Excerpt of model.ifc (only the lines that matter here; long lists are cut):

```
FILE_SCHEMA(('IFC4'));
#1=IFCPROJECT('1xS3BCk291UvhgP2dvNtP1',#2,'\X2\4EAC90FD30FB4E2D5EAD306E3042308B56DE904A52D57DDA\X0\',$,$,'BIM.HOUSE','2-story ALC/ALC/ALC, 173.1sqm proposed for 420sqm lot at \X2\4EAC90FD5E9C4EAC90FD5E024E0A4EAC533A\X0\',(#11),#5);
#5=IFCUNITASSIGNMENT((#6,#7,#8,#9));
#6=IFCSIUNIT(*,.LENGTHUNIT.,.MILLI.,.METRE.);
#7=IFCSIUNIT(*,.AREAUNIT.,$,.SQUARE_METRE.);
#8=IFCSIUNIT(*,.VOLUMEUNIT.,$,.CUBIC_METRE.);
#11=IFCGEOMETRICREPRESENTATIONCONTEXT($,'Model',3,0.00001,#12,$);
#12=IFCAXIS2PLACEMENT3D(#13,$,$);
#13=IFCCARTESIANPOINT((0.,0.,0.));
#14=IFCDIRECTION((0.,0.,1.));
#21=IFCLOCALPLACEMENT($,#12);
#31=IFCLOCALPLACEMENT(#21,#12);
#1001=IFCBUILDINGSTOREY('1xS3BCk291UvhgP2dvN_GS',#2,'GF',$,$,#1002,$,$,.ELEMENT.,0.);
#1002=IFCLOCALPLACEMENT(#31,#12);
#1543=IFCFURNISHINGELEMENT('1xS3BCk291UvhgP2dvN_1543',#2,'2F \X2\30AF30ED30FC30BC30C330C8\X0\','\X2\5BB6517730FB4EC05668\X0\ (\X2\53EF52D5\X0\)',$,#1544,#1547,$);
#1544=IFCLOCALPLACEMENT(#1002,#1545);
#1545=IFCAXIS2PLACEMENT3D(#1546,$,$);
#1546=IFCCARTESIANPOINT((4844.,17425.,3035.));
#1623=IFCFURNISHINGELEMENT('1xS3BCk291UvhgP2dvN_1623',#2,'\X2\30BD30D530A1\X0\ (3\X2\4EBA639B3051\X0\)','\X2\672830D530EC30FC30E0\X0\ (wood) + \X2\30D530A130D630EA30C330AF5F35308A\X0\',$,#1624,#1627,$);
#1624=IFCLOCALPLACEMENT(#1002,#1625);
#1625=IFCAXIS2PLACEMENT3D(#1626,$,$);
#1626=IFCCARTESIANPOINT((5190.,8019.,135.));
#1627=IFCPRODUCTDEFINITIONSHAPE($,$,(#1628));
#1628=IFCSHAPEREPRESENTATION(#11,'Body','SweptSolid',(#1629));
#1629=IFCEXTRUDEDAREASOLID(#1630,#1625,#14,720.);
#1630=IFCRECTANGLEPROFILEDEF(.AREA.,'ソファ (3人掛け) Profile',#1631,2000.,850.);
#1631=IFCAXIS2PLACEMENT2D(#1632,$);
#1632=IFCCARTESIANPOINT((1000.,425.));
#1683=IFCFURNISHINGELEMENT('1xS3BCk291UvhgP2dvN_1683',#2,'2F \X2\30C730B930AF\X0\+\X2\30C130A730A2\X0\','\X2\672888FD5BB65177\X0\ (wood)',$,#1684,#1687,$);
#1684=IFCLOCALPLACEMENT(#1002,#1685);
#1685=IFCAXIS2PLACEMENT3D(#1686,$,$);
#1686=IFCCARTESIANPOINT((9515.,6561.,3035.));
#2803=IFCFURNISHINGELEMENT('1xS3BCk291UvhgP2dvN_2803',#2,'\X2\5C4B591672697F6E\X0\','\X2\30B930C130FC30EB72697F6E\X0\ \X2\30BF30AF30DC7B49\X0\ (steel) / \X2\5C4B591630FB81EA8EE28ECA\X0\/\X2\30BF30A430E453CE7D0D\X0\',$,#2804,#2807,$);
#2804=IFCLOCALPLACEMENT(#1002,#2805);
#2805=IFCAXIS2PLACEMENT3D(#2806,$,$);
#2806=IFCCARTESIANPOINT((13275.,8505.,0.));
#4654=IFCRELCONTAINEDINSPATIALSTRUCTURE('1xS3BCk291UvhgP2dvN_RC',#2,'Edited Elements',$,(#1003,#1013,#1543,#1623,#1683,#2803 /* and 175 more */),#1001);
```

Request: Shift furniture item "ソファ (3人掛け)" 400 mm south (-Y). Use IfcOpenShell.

```python
import ifcopenshell
import ifcopenshell.api.geometry
import ifcopenshell.util.placement

model = ifcopenshell.open("model.ifc")

item = model.by_guid("1xS3BCk291UvhgP2dvN_1623")
matrix = ifcopenshell.util.placement.get_local_placement(item.ObjectPlacement)
matrix[1, 3] -= 400.0
ifcopenshell.api.geometry.edit_object_placement(model, product=item, matrix=matrix, is_si=False)

print(ifcopenshell.util.placement.get_local_placement(item.ObjectPlacement).round(3) + 0.0)

model.write("model_edited.ifc")
```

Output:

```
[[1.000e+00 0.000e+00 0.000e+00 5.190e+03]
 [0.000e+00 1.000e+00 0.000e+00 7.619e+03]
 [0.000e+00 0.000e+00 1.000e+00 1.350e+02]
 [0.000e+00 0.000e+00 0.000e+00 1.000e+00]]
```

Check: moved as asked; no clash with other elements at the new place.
